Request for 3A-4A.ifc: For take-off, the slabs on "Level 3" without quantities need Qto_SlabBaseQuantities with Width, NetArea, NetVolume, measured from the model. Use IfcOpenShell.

First a look at what the model holds.

```python
import ifcopenshell
import ifcopenshell.util.element
import ifcopenshell.util.unit

model = ifcopenshell.open("3A-4A.ifc")
print(model.schema)
for unit_type in ("LENGTHUNIT", "AREAUNIT", "VOLUMEUNIT"):
    print(unit_type, ifcopenshell.util.unit.calculate_unit_scale(model, unit_type))
storey = next(s for s in model.by_type("IfcBuildingStorey") if s.Name == "Level 3")
slabs = [e for e in ifcopenshell.util.element.get_decomposition(storey) if e.is_a("IfcSlab")]
for e in sorted(slabs, key=lambda e: e.id()):
    print(e.id(), e.is_a(), e.Name, list(ifcopenshell.util.element.get_psets(e, qtos_only=True)), sep=" | ")
```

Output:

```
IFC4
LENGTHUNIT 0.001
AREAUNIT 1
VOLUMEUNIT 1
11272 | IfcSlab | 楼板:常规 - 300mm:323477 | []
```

```python
import ifcopenshell
import ifcopenshell.api.pset
import ifcopenshell.geom
import ifcopenshell.util.element
import ifcopenshell.util.shape
import ifcopenshell.util.unit

model = ifcopenshell.open("3A-4A.ifc")
unit_scale = ifcopenshell.util.unit.calculate_unit_scale(model)
area_scale = ifcopenshell.util.unit.calculate_unit_scale(model, "AREAUNIT")
volume_scale = ifcopenshell.util.unit.calculate_unit_scale(model, "VOLUMEUNIT")
settings = ifcopenshell.geom.settings()

storey = next(s for s in model.by_type("IfcBuildingStorey") if s.Name == "Level 3")
slabs = [e for e in ifcopenshell.util.element.get_decomposition(storey) if e.is_a("IfcSlab")]

for e in sorted(slabs, key=lambda e: e.id()):
    if ifcopenshell.util.element.get_psets(e, qtos_only=True, should_inherit=False):
        continue
    # Geometry comes back in metres, in the element's own axes.
    shape = ifcopenshell.geom.create_shape(settings, e)
    values = {
        "Width": ifcopenshell.util.shape.get_z(shape.geometry) / unit_scale,
        "NetArea": ifcopenshell.util.shape.get_footprint_area(shape.geometry) / area_scale,
        "NetVolume": ifcopenshell.util.shape.get_volume(shape.geometry) / volume_scale,
    }
    qto = ifcopenshell.api.pset.add_qto(model, product=e, name="Qto_SlabBaseQuantities")
    ifcopenshell.api.pset.edit_qto(model, qto=qto, properties=values)
    print(e.id(), {k: round(v, 3) for k, v in values.items()})

model.write("3A-4A_v2.ifc")
```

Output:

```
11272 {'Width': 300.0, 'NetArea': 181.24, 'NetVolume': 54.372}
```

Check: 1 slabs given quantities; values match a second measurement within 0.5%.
